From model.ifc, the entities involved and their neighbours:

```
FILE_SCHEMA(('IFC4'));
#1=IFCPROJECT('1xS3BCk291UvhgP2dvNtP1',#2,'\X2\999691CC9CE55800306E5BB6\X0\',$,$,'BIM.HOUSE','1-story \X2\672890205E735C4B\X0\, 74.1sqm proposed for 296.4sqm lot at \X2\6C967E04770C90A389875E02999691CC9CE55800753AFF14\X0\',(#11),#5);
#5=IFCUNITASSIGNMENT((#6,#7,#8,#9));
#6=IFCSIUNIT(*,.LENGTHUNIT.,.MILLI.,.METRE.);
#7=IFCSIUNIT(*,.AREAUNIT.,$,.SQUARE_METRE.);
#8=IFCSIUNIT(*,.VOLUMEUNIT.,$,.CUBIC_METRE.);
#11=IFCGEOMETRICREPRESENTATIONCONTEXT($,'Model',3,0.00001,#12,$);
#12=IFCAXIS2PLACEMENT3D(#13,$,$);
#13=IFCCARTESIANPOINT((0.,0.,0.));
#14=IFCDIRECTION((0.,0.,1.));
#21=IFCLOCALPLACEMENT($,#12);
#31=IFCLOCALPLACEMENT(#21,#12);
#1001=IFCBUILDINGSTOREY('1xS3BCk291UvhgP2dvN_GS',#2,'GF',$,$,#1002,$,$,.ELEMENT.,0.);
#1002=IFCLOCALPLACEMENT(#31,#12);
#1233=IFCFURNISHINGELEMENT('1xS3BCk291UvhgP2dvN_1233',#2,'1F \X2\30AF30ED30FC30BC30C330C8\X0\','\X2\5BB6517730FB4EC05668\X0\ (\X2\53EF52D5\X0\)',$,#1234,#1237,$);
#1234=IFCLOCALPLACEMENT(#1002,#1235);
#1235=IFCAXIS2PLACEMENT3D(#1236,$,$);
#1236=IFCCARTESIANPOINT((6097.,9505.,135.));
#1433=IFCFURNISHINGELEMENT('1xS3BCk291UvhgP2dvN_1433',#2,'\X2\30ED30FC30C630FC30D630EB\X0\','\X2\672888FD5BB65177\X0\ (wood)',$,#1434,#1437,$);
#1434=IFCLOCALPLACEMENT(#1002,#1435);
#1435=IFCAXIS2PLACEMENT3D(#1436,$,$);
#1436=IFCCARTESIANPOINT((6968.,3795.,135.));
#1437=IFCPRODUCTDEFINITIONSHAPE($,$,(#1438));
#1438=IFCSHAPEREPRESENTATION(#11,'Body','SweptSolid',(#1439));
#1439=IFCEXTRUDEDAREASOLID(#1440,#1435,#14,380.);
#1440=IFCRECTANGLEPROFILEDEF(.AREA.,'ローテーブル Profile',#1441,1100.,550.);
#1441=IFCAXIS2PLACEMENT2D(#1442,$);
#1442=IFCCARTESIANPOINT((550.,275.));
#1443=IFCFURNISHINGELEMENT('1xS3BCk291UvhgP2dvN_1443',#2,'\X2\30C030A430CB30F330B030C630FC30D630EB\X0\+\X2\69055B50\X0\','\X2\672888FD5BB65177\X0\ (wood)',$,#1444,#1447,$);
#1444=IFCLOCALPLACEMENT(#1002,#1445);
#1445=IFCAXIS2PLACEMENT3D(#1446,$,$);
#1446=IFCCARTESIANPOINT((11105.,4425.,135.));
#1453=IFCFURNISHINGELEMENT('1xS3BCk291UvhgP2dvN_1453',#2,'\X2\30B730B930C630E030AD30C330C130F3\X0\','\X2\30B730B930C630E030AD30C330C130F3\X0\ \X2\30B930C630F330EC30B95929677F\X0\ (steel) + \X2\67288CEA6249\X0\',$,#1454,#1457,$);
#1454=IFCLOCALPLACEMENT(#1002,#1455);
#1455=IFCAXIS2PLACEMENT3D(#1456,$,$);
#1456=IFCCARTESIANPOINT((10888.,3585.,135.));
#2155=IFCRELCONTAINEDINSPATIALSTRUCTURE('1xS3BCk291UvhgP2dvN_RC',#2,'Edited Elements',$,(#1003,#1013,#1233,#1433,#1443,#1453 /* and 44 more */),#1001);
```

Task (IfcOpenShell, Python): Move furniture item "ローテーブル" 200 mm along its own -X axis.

```python
import ifcopenshell
import ifcopenshell.api.geometry
import ifcopenshell.util.placement

model = ifcopenshell.open("model.ifc")

item = model.by_guid("1xS3BCk291UvhgP2dvN_1433")
matrix = ifcopenshell.util.placement.get_local_placement(item.ObjectPlacement)
matrix[:3, 3] -= matrix[:3, 0] * 200.0
ifcopenshell.api.geometry.edit_object_placement(model, product=item, matrix=matrix, is_si=False)

print(ifcopenshell.util.placement.get_local_placement(item.ObjectPlacement).round(3) + 0.0)

model.write("model_updated.ifc")
```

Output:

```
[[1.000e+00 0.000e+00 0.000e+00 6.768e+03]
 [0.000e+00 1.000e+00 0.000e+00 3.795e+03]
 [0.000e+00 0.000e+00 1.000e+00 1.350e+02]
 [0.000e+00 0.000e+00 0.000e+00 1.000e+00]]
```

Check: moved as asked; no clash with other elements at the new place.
